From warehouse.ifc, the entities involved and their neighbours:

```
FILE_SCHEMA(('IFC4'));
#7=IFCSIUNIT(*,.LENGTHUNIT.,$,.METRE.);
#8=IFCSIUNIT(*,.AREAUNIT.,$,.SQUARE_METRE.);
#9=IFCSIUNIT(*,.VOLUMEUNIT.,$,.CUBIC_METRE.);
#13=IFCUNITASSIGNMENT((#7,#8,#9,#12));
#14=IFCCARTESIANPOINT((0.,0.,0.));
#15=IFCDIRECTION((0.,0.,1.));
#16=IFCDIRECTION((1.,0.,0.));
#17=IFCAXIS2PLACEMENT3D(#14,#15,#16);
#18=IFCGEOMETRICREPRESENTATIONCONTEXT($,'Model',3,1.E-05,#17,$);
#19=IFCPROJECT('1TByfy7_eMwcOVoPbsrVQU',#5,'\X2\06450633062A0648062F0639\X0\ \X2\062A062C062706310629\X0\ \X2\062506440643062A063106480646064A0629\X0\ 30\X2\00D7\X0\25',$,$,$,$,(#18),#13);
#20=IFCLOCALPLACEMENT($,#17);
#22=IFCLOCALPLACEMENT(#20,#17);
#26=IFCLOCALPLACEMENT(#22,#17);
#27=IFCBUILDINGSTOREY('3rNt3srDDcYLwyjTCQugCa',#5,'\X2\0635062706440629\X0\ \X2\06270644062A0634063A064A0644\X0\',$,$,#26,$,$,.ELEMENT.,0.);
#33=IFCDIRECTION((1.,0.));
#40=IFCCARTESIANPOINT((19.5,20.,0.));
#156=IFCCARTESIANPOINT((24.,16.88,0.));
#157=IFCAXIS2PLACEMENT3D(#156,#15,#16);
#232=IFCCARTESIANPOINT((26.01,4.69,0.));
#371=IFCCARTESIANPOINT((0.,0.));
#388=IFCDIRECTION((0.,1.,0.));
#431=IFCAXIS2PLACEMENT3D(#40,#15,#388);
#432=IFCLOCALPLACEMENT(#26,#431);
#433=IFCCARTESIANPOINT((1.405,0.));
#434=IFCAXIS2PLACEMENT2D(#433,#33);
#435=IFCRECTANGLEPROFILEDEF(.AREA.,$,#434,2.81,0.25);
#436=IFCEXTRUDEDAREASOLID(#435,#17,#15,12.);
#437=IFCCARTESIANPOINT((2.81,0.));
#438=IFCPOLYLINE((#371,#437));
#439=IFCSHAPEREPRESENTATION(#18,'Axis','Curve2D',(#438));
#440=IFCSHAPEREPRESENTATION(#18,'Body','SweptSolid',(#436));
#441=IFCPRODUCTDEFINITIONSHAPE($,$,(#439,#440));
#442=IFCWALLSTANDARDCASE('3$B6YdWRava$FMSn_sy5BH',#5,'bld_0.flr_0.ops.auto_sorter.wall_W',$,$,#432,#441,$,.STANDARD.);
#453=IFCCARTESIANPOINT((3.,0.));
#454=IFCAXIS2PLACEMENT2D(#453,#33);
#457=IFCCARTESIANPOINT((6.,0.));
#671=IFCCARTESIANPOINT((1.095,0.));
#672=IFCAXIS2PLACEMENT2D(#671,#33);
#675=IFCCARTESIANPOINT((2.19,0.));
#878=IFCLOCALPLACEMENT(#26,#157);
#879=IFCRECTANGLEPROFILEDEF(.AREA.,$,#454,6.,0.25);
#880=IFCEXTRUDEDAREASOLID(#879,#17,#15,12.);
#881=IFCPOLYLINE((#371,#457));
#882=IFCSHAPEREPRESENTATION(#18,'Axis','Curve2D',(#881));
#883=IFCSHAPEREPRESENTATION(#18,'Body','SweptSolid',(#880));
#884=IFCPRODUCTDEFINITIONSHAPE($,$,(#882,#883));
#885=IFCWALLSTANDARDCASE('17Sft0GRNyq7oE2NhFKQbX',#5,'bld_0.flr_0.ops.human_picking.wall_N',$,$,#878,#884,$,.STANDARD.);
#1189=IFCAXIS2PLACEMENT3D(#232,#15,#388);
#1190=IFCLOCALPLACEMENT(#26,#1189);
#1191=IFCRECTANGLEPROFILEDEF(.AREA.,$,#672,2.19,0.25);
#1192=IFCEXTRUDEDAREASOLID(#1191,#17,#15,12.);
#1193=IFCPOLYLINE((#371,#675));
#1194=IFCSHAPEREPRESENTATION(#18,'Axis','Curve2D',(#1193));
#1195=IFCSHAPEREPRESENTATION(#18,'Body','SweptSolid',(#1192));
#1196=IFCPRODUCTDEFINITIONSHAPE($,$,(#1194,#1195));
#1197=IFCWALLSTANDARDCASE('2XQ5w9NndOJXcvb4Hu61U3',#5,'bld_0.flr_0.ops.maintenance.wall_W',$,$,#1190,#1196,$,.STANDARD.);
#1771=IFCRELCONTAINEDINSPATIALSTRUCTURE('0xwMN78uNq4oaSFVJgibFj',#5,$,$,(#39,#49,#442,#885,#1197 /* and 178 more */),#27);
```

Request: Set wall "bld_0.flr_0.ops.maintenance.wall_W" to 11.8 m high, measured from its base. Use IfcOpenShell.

```python
import ifcopenshell
import ifcopenshell.geom
import ifcopenshell.util.shape
import ifcopenshell.util.unit

model = ifcopenshell.open("warehouse.ifc")
unit_scale = ifcopenshell.util.unit.calculate_unit_scale(model)
settings = ifcopenshell.geom.settings()


def volume(element):
    """Net volume in cubic metres, openings subtracted."""
    shape = ifcopenshell.geom.create_shape(settings, element)
    return ifcopenshell.util.shape.get_volume(shape.geometry)


wall = model.by_id(1197)
before = volume(wall)

body = next(r for r in wall.Representation.Representations if r.RepresentationIdentifier == "Body")
solid = body.Items[0]
old_height = solid.Depth
solid.Depth = 11.8 / unit_scale
after = volume(wall)

print(f"height {old_height:g} -> {solid.Depth:g}, volume {before:.3f} -> {after:.3f} m3")

model.write("warehouse_v2.ifc")
```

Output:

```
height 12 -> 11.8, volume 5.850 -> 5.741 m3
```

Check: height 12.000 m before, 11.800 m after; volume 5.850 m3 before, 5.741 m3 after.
